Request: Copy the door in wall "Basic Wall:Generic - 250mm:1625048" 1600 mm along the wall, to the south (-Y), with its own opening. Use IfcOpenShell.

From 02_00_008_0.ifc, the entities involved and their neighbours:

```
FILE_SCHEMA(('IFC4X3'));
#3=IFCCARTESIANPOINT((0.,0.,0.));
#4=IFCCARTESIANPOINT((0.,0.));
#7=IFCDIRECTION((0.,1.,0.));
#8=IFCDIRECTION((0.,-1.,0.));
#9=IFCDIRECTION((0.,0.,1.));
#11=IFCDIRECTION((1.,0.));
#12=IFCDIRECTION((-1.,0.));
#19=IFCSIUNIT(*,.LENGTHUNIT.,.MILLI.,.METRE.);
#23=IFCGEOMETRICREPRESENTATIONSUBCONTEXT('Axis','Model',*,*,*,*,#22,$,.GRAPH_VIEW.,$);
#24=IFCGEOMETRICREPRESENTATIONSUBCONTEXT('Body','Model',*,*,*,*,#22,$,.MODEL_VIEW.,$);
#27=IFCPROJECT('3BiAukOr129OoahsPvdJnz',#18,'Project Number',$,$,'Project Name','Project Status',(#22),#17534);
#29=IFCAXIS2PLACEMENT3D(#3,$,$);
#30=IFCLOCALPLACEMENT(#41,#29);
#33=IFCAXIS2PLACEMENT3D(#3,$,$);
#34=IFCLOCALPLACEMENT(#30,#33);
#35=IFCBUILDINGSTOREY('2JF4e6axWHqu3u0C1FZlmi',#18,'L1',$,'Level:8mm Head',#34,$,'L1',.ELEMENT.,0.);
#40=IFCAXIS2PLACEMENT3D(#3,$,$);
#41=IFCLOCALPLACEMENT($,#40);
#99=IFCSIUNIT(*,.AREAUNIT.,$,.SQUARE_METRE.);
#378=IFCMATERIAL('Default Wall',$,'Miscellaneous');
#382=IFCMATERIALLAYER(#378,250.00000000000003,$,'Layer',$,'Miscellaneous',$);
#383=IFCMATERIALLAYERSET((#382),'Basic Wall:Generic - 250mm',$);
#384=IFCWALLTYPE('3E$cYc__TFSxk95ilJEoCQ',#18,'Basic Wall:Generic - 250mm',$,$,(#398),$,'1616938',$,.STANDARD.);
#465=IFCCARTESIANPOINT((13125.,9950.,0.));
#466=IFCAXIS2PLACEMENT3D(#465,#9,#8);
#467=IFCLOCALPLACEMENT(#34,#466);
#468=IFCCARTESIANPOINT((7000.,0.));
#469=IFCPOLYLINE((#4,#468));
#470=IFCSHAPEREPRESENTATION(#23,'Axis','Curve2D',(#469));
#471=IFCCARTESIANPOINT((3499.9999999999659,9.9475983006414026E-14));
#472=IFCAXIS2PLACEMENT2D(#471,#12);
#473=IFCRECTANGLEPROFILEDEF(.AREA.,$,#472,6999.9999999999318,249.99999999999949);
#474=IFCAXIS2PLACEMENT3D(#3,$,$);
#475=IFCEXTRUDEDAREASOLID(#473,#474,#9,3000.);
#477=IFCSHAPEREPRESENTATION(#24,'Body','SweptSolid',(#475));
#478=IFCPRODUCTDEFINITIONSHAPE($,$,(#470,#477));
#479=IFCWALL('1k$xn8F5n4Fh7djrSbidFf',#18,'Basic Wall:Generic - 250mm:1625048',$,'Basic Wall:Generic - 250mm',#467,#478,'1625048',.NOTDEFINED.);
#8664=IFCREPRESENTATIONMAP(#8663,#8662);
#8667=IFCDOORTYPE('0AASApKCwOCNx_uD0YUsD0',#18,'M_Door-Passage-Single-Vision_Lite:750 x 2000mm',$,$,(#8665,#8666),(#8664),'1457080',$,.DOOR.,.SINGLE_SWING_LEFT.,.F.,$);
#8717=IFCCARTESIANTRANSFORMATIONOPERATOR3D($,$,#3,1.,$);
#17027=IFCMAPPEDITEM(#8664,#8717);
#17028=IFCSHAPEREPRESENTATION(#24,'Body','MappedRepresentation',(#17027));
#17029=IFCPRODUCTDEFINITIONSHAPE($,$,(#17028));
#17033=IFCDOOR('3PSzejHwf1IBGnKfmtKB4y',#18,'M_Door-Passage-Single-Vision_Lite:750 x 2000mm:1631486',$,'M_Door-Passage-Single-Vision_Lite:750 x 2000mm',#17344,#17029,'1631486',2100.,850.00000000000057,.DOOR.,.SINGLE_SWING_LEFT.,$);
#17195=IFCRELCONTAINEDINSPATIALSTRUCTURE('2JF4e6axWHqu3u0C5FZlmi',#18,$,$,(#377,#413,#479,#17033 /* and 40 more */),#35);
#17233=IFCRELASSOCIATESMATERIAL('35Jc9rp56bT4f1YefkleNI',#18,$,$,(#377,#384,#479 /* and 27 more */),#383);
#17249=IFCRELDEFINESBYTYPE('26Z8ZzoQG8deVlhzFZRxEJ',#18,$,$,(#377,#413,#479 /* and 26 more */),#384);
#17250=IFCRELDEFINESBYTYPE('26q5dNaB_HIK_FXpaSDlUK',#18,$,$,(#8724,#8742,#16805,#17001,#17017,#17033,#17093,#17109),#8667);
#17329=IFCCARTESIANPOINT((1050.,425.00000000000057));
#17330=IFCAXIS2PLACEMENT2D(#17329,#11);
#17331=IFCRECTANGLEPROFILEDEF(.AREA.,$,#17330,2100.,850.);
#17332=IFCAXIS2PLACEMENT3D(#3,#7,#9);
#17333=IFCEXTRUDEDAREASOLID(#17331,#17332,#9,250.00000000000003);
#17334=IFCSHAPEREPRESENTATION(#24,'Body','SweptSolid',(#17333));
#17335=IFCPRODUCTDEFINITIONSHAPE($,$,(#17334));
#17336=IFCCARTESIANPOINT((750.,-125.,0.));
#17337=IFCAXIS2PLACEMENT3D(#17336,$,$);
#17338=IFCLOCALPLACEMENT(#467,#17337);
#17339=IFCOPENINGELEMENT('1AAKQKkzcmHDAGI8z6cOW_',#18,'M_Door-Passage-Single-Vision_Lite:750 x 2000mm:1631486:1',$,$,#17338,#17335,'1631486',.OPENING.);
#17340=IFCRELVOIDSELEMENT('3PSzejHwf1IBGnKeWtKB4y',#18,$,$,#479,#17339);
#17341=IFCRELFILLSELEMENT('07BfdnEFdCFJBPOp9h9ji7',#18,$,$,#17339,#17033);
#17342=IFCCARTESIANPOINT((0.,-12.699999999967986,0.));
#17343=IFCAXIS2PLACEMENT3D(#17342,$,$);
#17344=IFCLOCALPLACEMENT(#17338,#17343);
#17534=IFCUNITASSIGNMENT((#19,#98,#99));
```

```python
import ifcopenshell
import ifcopenshell.api.feature
import ifcopenshell.api.geometry
import ifcopenshell.api.root
import ifcopenshell.geom
import ifcopenshell.util.element
import ifcopenshell.util.placement
import ifcopenshell.util.shape

model = ifcopenshell.open("02_00_008_0.ifc")
settings = ifcopenshell.geom.settings()


def volume(element):
    """Net volume in cubic metres, openings subtracted."""
    shape = ifcopenshell.geom.create_shape(settings, element)
    return ifcopenshell.util.shape.get_volume(shape.geometry)


def reuse_history(source, copy):
    """copy_class also copies each property set's owner history, people and application; keep the originals."""
    for rel in copy.IsDefinedBy:
        if rel.is_a("IfcRelDefinesByProperties") and (history := rel.RelatingPropertyDefinition.OwnerHistory):
            rel.RelatingPropertyDefinition.OwnerHistory = source.OwnerHistory
            ifcopenshell.util.element.remove_deep2(model, history)


door = model.by_guid("3PSzejHwf1IBGnKfmtKB4y")
opening = door.FillsVoids[0].RelatingOpeningElement
wall = opening.VoidsElements[0].RelatingBuildingElement
before = volume(wall)
shift = ifcopenshell.util.placement.get_local_placement(wall.ObjectPlacement)[:3, 0] * 1600.0

# copy_class copies the void relationship, type, container and properties, but no geometry.
new_opening = ifcopenshell.api.root.copy_class(model, product=opening)
new_opening.Representation = ifcopenshell.util.element.copy_deep(
    model, opening.Representation, exclude=["IfcGeometricRepresentationContext", "IfcRepresentationMap"]
)
new_opening.Name = "M_Door-Passage-Single-Vision_Lite:750 x 2000mm"
new_opening.Tag = None
new_door = ifcopenshell.api.root.copy_class(model, product=door)
new_door.Representation = ifcopenshell.util.element.copy_deep(
    model, door.Representation, exclude=["IfcGeometricRepresentationContext", "IfcRepresentationMap"]
)
new_door.Name = "M_Door-Passage-Single-Vision_Lite:750 x 2000mm"
new_door.Tag = None
reuse_history(door, new_door)
ifcopenshell.api.feature.add_filling(model, opening=new_opening, element=new_door)

for old, new in ((opening, new_opening), (door, new_door)):
    matrix = ifcopenshell.util.placement.get_local_placement(old.ObjectPlacement)
    matrix[:3, 3] += shift
    ifcopenshell.api.geometry.edit_object_placement(model, product=new, matrix=matrix, is_si=False)

after = volume(wall)

print(f"wall volume {before:.3f} -> {after:.3f} m3")

model.write("02_00_008_0-out.ifc")
```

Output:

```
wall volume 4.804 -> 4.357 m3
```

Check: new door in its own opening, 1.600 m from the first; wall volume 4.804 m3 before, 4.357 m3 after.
